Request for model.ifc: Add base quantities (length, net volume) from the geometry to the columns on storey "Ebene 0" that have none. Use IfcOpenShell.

First a look at what the model holds.

```python
import ifcopenshell
import ifcopenshell.util.element
import ifcopenshell.util.unit

model = ifcopenshell.open("model.ifc")
print(model.schema)
for unit_type in ("LENGTHUNIT", "AREAUNIT", "VOLUMEUNIT"):
    print(unit_type, ifcopenshell.util.unit.calculate_unit_scale(model, unit_type))
storey = next(s for s in model.by_type("IfcBuildingStorey") if s.Name == "Ebene 0")
columns = [e for e in ifcopenshell.util.element.get_decomposition(storey) if e.is_a("IfcColumn")]
for e in sorted(columns, key=lambda e: e.id()):
    print(e.id(), e.is_a(), e.Name, list(ifcopenshell.util.element.get_psets(e, qtos_only=True)), sep=" | ")
```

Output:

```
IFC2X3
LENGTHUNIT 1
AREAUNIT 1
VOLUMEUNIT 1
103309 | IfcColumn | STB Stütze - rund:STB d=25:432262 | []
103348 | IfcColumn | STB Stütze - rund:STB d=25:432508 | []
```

```python
import ifcopenshell
import ifcopenshell.api.pset
import ifcopenshell.geom
import ifcopenshell.util.element
import ifcopenshell.util.shape
import ifcopenshell.util.unit

model = ifcopenshell.open("model.ifc")
unit_scale = ifcopenshell.util.unit.calculate_unit_scale(model)
volume_scale = ifcopenshell.util.unit.calculate_unit_scale(model, "VOLUMEUNIT")
settings = ifcopenshell.geom.settings()

storey = next(s for s in model.by_type("IfcBuildingStorey") if s.Name == "Ebene 0")
columns = [e for e in ifcopenshell.util.element.get_decomposition(storey) if e.is_a("IfcColumn")]

for e in sorted(columns, key=lambda e: e.id()):
    if ifcopenshell.util.element.get_psets(e, qtos_only=True, should_inherit=False):
        continue
    # Geometry comes back in metres, in the element's own axes.
    shape = ifcopenshell.geom.create_shape(settings, e)
    values = {
        "Length": ifcopenshell.util.shape.get_z(shape.geometry) / unit_scale,
        "NetVolume": ifcopenshell.util.shape.get_volume(shape.geometry) / volume_scale,
    }
    qto = ifcopenshell.api.pset.add_qto(model, product=e, name="BaseQuantities")
    ifcopenshell.api.pset.edit_qto(model, qto=qto, properties=values)
    print(e.id(), {k: round(v, 3) for k, v in values.items()})

model.write("model_v2.ifc")
```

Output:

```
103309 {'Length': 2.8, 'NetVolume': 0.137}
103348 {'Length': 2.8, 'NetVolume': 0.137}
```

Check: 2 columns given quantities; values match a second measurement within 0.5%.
